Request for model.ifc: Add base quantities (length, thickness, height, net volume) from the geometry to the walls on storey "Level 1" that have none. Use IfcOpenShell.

First a look at what the model holds.

```python
import ifcopenshell
import ifcopenshell.util.element
import ifcopenshell.util.unit

model = ifcopenshell.open("model.ifc")
print(model.schema)
for unit_type in ("LENGTHUNIT", "AREAUNIT", "VOLUMEUNIT"):
    print(unit_type, ifcopenshell.util.unit.calculate_unit_scale(model, unit_type))
storey = next(s for s in model.by_type("IfcBuildingStorey") if s.Name == "Level 1")
walls = [e for e in ifcopenshell.util.element.get_decomposition(storey) if e.is_a("IfcWall")]
for e in sorted(walls, key=lambda e: e.id()):
    print(e.id(), e.is_a(), e.Name, list(ifcopenshell.util.element.get_psets(e, qtos_only=True)), sep=" | ")
```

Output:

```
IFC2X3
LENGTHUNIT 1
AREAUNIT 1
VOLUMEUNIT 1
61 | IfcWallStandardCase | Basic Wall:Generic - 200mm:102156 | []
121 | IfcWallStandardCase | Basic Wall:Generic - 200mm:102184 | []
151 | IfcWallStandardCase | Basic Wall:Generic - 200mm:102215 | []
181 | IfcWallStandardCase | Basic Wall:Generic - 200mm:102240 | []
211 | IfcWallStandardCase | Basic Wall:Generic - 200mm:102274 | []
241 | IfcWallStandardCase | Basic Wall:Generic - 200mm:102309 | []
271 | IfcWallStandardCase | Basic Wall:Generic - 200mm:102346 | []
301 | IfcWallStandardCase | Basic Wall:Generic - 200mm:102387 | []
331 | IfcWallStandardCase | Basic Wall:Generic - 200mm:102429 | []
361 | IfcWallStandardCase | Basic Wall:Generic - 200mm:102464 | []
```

```python
import ifcopenshell
import ifcopenshell.api.pset
import ifcopenshell.geom
import ifcopenshell.util.element
import ifcopenshell.util.shape
import ifcopenshell.util.unit

model = ifcopenshell.open("model.ifc")
unit_scale = ifcopenshell.util.unit.calculate_unit_scale(model)
volume_scale = ifcopenshell.util.unit.calculate_unit_scale(model, "VOLUMEUNIT")
settings = ifcopenshell.geom.settings()

storey = next(s for s in model.by_type("IfcBuildingStorey") if s.Name == "Level 1")
walls = [e for e in ifcopenshell.util.element.get_decomposition(storey) if e.is_a("IfcWall")]

for e in sorted(walls, key=lambda e: e.id()):
    if ifcopenshell.util.element.get_psets(e, qtos_only=True, should_inherit=False):
        continue
    # Geometry comes back in metres, in the element's own axes.
    shape = ifcopenshell.geom.create_shape(settings, e)
    values = {
        "Length": ifcopenshell.util.shape.get_x(shape.geometry) / unit_scale,
        "Width": ifcopenshell.util.shape.get_y(shape.geometry) / unit_scale,
        "Height": ifcopenshell.util.shape.get_z(shape.geometry) / unit_scale,
        "NetVolume": ifcopenshell.util.shape.get_volume(shape.geometry) / volume_scale,
    }
    qto = ifcopenshell.api.pset.add_qto(model, product=e, name="BaseQuantities")
    ifcopenshell.api.pset.edit_qto(model, qto=qto, properties=values)
    print(e.id(), {k: round(v, 3) for k, v in values.items()})

model.write("model_updated.ifc")
```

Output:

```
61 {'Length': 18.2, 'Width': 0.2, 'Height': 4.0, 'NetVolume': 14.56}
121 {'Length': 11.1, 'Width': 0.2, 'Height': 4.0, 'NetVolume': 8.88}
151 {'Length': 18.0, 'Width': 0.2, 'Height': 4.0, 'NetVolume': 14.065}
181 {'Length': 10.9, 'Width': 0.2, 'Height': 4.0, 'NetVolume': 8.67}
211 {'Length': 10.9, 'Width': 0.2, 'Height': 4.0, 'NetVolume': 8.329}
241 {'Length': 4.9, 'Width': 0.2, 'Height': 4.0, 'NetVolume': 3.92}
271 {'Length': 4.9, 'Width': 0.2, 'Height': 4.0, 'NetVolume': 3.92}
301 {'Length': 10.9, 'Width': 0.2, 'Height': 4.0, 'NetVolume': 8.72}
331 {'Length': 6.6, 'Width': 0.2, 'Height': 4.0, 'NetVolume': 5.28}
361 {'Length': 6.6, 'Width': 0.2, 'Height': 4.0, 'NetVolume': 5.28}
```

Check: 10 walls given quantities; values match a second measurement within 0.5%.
